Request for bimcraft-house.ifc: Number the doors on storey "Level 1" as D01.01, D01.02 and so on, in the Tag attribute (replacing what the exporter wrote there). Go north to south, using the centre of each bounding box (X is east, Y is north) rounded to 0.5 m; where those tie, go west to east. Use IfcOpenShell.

First a look at what the model holds.

```python
import ifcopenshell
import ifcopenshell.util.element
import ifcopenshell.util.placement

model = ifcopenshell.open("bimcraft-house.ifc")
print(model.schema)
storey = next(s for s in model.by_type("IfcBuildingStorey") if s.Name == "Level 1")
doors = [e for e in ifcopenshell.util.element.get_decomposition(storey) if e.is_a("IfcDoor")]
for e in sorted(doors, key=lambda e: e.id()):
    origin = ifcopenshell.util.placement.get_local_placement(e.ObjectPlacement)[:3, 3]
    print(e.id(), e.Tag, e.Name, origin.round(2) + 0.0, sep=" | ")
```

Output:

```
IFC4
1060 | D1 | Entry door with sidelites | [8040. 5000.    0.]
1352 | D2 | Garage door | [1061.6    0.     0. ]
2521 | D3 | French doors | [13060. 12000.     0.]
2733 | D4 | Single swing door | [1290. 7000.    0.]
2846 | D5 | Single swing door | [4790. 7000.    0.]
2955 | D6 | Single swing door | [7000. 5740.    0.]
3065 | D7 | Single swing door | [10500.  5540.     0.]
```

```python
import ifcopenshell
import ifcopenshell.geom
import ifcopenshell.util.element
import ifcopenshell.util.shape

model = ifcopenshell.open("bimcraft-house.ifc")
settings = ifcopenshell.geom.settings()
settings.set("use-world-coords", True)


def centre(element):
    shape = ifcopenshell.geom.create_shape(settings, element)
    return ifcopenshell.util.shape.get_bbox_centroid(shape.geometry)


storey = next(s for s in model.by_type("IfcBuildingStorey") if s.Name == "Level 1")
doors = [e for e in ifcopenshell.util.element.get_decomposition(storey) if e.is_a("IfcDoor")]

# Insertion points can sit at a corner or the storey origin, so sort by the geometry (in metres).
centres = {e: centre(e) for e in doors}
doors.sort(key=lambda e: (-round(centres[e][1] / 0.5), centres[e][0]))

for i, e in enumerate(doors, start=1):
    number = f"D01.{i:02d}"
    e.Tag = number
    print(e.id(), number)

model.write("bimcraft-house-out.ifc")
```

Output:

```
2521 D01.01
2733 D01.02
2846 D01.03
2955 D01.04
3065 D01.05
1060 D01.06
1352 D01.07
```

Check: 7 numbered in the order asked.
